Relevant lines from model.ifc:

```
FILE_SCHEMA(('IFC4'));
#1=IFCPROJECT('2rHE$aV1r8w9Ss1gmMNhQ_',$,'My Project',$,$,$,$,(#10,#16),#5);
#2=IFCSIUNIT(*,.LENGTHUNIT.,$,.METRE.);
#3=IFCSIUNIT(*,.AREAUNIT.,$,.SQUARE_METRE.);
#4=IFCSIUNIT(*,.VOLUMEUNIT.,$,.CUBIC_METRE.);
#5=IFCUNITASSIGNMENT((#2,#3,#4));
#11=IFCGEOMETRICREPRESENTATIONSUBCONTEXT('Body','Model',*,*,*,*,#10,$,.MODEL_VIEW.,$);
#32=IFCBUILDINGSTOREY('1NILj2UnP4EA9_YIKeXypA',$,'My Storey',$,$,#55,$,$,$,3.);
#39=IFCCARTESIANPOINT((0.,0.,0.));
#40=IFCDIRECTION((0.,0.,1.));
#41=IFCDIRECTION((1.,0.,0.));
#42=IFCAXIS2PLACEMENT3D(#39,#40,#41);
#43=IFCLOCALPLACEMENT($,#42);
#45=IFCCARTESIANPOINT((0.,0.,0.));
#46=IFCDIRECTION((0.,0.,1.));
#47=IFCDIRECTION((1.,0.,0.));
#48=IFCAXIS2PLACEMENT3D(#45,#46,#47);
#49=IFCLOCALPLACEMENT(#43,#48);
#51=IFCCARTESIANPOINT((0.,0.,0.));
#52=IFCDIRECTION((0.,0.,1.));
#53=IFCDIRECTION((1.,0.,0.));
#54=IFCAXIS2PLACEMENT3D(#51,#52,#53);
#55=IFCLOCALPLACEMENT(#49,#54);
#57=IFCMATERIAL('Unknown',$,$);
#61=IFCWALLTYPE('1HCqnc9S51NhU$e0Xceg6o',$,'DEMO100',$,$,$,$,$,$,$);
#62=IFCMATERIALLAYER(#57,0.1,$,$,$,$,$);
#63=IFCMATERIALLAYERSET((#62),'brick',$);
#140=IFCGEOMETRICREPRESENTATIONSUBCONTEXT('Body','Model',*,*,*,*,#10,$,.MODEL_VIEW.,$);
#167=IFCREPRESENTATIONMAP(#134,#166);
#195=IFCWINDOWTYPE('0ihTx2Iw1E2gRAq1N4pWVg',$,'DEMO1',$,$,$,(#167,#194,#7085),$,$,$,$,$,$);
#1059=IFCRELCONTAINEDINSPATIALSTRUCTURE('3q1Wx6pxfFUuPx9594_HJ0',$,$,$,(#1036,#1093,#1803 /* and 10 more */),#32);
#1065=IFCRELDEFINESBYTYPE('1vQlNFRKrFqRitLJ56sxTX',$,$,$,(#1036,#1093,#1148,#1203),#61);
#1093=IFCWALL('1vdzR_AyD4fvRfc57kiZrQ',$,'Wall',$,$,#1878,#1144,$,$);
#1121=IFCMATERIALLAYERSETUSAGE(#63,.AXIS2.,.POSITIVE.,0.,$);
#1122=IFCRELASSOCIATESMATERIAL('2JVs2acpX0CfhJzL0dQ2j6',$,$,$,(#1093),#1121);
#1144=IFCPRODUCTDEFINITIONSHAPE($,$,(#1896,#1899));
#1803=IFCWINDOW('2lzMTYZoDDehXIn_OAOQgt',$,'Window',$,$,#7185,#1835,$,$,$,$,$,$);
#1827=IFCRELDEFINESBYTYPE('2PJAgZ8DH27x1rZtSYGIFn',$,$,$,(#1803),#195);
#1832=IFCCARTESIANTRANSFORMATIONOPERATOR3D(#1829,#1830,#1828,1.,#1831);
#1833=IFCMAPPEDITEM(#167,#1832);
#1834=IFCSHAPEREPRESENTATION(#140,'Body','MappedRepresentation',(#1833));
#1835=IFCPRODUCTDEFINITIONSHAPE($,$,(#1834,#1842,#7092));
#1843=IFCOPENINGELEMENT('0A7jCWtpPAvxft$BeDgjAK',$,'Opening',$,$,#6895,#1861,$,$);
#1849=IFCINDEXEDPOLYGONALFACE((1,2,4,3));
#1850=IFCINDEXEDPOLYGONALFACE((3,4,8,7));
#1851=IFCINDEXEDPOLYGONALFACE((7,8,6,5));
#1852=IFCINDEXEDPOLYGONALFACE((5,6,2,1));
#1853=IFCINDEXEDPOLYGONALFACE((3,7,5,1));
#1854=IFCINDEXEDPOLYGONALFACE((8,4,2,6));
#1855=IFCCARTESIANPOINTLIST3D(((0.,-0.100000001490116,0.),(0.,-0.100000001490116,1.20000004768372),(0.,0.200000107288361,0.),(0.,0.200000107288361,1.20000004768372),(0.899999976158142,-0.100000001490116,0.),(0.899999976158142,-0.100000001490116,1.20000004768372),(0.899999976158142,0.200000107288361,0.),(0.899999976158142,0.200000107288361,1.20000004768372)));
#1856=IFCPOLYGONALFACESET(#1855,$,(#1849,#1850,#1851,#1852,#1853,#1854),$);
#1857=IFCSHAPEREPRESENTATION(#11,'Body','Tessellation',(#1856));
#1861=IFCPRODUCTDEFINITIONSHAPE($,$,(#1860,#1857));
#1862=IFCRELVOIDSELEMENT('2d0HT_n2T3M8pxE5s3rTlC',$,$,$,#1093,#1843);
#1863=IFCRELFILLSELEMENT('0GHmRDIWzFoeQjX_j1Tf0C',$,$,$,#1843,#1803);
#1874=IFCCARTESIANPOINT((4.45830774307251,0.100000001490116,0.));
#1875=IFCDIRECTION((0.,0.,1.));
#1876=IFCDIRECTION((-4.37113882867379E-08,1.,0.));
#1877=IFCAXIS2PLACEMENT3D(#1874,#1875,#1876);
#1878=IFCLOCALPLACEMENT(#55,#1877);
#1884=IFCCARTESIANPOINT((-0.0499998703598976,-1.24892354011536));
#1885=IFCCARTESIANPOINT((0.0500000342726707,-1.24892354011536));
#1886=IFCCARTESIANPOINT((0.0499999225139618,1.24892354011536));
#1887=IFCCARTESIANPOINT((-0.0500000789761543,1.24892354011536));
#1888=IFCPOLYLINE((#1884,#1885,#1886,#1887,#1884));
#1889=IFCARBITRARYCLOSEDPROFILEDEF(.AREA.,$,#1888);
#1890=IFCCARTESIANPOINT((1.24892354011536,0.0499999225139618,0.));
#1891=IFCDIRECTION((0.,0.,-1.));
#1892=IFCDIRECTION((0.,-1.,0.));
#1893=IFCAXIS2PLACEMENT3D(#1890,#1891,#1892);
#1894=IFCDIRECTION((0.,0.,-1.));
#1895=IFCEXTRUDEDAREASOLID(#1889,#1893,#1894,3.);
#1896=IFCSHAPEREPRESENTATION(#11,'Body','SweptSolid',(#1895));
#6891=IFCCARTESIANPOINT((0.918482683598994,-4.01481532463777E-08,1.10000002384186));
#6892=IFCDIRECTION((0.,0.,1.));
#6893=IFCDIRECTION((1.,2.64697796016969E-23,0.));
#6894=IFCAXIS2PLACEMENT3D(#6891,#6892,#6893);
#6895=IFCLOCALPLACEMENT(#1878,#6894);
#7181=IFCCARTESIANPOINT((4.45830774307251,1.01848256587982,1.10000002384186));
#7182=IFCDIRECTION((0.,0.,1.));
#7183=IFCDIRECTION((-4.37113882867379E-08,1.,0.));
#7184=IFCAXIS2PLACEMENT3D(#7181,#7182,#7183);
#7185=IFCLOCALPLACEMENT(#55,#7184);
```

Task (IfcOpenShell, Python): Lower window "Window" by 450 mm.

```python
import numpy as np
import ifcopenshell
import ifcopenshell.api.geometry
import ifcopenshell.util.placement
import ifcopenshell.util.unit

model = ifcopenshell.open("model.ifc")
unit_scale = ifcopenshell.util.unit.calculate_unit_scale(model)

window = model.by_guid("2lzMTYZoDDehXIn_OAOQgt")
opening = window.FillsVoids[0].RelatingOpeningElement
dz = -0.45

shift = np.array([0.0, 0.0, dz])
# The window is not placed relative to its opening, so move both.
for product in (opening, window):
    matrix = ifcopenshell.util.placement.get_local_placement(product.ObjectPlacement)
    matrix[:3, 3] += shift
    ifcopenshell.api.geometry.edit_object_placement(model, product=product, matrix=matrix, is_si=False)

print(f"moved by {dz * unit_scale:+.3f} m")

model.write("model_updated.ifc")
```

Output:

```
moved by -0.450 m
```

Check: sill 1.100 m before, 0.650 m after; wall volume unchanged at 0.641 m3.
